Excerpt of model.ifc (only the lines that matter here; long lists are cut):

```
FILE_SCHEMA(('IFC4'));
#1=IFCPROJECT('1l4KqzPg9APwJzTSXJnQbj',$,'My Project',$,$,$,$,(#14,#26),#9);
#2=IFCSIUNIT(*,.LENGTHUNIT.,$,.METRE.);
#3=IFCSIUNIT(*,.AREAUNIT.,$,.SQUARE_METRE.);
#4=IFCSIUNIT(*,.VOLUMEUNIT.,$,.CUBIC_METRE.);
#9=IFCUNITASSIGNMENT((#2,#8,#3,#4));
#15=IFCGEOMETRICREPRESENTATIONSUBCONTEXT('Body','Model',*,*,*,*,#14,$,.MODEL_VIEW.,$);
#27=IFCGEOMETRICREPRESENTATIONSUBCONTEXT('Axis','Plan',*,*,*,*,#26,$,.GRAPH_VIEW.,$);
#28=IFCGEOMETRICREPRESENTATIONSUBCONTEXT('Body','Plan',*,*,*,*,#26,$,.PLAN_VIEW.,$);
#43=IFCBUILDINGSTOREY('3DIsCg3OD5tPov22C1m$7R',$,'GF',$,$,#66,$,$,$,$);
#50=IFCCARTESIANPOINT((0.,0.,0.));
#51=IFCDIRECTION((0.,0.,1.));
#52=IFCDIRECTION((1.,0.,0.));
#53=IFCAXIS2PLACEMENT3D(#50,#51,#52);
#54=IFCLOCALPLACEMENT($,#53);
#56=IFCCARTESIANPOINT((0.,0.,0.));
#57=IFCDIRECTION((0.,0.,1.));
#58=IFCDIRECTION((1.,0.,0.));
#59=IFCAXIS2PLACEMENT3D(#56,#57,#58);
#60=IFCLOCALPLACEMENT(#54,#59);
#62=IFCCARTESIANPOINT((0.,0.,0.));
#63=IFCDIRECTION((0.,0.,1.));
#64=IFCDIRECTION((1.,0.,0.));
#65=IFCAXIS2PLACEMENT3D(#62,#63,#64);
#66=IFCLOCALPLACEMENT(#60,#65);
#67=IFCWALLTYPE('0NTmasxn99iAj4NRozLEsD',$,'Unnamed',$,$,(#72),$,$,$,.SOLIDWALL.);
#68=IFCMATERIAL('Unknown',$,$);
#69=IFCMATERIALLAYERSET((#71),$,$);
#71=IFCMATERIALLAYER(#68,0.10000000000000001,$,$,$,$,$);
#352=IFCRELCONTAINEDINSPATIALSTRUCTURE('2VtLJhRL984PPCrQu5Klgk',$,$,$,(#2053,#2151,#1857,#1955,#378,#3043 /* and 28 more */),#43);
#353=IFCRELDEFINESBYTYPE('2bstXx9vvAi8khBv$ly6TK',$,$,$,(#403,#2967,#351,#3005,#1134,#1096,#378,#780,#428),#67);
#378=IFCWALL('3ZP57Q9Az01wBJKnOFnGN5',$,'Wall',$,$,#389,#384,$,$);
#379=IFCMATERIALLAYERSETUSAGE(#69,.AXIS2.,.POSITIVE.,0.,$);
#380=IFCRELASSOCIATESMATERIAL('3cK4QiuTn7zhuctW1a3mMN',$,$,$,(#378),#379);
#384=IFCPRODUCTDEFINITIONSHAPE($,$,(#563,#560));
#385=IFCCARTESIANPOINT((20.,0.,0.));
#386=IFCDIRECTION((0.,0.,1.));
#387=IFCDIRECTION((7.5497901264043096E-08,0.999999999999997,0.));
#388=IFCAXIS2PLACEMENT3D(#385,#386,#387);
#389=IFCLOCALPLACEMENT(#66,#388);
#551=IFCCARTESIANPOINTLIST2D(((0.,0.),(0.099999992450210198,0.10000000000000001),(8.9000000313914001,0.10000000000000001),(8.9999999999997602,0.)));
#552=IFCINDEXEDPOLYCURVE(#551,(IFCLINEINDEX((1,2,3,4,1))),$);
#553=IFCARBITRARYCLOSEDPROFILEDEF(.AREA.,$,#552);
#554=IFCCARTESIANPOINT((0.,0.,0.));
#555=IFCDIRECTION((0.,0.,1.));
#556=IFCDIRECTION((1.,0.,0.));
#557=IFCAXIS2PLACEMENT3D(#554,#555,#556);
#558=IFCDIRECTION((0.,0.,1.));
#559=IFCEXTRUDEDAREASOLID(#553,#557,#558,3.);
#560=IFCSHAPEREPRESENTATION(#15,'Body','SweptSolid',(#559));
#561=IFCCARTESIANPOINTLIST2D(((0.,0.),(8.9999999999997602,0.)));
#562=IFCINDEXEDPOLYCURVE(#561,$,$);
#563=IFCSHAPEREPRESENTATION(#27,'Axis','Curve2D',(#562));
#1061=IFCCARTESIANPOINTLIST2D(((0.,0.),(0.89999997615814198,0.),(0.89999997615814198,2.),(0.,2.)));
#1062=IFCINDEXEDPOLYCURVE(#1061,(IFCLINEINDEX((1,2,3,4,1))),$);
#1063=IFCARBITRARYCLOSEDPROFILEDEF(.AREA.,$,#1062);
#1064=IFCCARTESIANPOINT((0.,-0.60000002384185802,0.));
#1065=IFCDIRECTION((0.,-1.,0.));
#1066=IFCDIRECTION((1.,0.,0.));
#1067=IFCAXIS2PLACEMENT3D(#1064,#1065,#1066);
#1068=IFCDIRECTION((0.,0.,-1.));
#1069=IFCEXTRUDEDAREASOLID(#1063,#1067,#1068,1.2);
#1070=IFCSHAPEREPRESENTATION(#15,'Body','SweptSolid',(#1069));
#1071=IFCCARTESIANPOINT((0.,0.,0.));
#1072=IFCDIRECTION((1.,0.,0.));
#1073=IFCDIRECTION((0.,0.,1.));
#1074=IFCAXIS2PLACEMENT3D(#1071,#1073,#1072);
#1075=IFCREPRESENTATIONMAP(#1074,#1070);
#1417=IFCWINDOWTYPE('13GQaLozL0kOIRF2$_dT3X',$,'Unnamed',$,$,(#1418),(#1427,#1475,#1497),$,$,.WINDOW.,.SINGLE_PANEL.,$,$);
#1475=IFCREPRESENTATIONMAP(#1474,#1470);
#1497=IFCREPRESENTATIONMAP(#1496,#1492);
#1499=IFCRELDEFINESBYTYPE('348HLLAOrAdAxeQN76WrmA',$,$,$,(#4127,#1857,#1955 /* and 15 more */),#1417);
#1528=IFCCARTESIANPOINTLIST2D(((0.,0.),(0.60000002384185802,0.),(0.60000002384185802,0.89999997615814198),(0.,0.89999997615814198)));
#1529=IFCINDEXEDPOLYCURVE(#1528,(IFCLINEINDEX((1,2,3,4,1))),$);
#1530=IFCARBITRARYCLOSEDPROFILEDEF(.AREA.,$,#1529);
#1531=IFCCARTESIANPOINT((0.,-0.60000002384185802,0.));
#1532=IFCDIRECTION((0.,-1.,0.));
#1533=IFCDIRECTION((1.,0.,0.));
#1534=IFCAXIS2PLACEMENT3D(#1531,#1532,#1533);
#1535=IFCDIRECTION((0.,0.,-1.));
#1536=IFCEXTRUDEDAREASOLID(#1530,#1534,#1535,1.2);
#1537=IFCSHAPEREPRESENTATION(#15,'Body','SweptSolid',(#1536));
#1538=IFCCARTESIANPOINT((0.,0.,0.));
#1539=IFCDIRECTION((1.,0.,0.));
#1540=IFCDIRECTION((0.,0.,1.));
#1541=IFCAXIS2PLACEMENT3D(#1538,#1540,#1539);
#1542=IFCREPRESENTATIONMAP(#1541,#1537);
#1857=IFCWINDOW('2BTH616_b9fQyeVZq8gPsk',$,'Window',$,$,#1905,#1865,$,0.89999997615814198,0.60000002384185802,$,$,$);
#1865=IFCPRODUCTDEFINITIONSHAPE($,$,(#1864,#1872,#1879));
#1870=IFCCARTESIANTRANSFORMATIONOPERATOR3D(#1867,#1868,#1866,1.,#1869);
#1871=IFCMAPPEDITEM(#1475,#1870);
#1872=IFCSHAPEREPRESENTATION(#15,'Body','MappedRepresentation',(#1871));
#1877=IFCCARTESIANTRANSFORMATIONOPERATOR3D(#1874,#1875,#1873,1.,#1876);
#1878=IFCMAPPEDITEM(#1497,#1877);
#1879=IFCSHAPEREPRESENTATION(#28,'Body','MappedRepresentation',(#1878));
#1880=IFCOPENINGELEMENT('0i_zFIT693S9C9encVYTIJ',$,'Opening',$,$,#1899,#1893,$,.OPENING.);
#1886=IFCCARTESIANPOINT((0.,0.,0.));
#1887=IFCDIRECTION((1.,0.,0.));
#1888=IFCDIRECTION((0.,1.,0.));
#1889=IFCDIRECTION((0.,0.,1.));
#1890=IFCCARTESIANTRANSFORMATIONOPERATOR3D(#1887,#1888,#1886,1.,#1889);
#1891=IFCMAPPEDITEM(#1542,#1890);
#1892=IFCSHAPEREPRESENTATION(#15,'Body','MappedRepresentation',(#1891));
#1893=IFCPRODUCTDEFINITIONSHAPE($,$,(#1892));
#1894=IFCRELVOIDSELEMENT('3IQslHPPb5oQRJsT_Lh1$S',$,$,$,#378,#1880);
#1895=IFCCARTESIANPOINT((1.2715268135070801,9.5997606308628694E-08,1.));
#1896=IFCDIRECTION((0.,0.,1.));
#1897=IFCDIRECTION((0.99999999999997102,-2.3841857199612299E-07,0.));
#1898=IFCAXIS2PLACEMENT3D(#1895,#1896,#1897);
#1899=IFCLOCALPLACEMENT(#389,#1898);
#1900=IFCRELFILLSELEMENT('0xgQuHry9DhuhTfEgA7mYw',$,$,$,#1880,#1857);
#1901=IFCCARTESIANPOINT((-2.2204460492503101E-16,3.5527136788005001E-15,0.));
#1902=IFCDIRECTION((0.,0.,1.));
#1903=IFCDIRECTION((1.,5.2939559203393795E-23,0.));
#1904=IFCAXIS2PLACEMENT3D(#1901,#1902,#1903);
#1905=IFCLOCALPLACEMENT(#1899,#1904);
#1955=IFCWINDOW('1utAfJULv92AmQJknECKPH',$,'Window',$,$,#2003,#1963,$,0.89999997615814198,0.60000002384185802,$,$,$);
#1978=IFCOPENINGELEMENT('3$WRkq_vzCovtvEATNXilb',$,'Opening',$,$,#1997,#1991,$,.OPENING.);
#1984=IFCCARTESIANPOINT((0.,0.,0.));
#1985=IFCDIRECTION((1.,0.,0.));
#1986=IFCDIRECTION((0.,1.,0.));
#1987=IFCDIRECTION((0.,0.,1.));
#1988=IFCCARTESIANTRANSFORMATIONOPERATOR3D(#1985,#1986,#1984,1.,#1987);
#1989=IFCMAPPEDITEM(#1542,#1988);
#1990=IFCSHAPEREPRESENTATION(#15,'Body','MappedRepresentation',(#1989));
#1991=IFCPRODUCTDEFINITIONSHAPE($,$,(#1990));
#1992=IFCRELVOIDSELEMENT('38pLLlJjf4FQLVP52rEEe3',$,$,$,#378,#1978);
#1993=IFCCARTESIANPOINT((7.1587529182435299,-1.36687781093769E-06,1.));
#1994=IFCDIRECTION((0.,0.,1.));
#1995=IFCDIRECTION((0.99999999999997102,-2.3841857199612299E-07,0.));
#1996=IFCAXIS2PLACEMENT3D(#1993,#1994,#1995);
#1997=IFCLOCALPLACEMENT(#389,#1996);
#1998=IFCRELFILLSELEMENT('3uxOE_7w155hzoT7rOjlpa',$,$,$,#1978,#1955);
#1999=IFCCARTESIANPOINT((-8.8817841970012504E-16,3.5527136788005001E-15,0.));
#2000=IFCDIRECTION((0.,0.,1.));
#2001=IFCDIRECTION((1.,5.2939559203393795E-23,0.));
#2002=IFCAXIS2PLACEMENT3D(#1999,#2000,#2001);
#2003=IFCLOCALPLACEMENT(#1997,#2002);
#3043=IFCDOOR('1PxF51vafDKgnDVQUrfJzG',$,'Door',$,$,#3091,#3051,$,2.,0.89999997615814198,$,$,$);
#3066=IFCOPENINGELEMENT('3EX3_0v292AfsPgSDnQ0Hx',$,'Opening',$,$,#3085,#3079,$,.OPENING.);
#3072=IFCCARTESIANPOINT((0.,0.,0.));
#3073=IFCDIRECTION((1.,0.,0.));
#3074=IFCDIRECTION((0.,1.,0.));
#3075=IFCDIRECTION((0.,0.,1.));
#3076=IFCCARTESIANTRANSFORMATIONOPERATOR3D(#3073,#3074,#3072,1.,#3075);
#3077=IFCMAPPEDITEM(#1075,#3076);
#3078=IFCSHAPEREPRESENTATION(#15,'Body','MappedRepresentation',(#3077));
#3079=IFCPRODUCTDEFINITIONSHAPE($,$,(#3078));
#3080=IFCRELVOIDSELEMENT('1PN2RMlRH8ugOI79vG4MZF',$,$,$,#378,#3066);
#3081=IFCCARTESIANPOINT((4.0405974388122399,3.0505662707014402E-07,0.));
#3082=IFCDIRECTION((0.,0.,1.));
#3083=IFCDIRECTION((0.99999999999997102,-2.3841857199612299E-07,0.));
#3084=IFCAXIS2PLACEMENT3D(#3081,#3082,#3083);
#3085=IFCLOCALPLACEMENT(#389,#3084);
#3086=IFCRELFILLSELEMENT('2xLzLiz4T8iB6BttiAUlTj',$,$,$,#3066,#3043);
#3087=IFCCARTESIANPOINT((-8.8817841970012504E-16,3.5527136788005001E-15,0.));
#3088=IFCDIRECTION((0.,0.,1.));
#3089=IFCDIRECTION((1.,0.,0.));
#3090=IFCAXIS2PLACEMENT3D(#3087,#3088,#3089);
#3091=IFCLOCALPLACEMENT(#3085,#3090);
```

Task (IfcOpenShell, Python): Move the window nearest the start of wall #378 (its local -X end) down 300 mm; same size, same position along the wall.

```python
import numpy as np
import ifcopenshell
import ifcopenshell.api.geometry
import ifcopenshell.util.placement
import ifcopenshell.util.unit

model = ifcopenshell.open("model.ifc")
unit_scale = ifcopenshell.util.unit.calculate_unit_scale(model)

window = model.by_id(1857)
opening = window.FillsVoids[0].RelatingOpeningElement
dz = -0.3 / unit_scale

shift = np.array([0.0, 0.0, dz])
# The window is placed relative to its opening, so it follows when the opening moves.
matrix = ifcopenshell.util.placement.get_local_placement(opening.ObjectPlacement)
matrix[:3, 3] += shift
ifcopenshell.api.geometry.edit_object_placement(
    model, product=opening, matrix=matrix, is_si=False, should_transform_children=True
)

print(f"moved by {dz * unit_scale:+.3f} m")

model.write("model_updated.ifc")
```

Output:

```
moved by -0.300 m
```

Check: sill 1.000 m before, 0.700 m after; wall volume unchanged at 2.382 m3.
